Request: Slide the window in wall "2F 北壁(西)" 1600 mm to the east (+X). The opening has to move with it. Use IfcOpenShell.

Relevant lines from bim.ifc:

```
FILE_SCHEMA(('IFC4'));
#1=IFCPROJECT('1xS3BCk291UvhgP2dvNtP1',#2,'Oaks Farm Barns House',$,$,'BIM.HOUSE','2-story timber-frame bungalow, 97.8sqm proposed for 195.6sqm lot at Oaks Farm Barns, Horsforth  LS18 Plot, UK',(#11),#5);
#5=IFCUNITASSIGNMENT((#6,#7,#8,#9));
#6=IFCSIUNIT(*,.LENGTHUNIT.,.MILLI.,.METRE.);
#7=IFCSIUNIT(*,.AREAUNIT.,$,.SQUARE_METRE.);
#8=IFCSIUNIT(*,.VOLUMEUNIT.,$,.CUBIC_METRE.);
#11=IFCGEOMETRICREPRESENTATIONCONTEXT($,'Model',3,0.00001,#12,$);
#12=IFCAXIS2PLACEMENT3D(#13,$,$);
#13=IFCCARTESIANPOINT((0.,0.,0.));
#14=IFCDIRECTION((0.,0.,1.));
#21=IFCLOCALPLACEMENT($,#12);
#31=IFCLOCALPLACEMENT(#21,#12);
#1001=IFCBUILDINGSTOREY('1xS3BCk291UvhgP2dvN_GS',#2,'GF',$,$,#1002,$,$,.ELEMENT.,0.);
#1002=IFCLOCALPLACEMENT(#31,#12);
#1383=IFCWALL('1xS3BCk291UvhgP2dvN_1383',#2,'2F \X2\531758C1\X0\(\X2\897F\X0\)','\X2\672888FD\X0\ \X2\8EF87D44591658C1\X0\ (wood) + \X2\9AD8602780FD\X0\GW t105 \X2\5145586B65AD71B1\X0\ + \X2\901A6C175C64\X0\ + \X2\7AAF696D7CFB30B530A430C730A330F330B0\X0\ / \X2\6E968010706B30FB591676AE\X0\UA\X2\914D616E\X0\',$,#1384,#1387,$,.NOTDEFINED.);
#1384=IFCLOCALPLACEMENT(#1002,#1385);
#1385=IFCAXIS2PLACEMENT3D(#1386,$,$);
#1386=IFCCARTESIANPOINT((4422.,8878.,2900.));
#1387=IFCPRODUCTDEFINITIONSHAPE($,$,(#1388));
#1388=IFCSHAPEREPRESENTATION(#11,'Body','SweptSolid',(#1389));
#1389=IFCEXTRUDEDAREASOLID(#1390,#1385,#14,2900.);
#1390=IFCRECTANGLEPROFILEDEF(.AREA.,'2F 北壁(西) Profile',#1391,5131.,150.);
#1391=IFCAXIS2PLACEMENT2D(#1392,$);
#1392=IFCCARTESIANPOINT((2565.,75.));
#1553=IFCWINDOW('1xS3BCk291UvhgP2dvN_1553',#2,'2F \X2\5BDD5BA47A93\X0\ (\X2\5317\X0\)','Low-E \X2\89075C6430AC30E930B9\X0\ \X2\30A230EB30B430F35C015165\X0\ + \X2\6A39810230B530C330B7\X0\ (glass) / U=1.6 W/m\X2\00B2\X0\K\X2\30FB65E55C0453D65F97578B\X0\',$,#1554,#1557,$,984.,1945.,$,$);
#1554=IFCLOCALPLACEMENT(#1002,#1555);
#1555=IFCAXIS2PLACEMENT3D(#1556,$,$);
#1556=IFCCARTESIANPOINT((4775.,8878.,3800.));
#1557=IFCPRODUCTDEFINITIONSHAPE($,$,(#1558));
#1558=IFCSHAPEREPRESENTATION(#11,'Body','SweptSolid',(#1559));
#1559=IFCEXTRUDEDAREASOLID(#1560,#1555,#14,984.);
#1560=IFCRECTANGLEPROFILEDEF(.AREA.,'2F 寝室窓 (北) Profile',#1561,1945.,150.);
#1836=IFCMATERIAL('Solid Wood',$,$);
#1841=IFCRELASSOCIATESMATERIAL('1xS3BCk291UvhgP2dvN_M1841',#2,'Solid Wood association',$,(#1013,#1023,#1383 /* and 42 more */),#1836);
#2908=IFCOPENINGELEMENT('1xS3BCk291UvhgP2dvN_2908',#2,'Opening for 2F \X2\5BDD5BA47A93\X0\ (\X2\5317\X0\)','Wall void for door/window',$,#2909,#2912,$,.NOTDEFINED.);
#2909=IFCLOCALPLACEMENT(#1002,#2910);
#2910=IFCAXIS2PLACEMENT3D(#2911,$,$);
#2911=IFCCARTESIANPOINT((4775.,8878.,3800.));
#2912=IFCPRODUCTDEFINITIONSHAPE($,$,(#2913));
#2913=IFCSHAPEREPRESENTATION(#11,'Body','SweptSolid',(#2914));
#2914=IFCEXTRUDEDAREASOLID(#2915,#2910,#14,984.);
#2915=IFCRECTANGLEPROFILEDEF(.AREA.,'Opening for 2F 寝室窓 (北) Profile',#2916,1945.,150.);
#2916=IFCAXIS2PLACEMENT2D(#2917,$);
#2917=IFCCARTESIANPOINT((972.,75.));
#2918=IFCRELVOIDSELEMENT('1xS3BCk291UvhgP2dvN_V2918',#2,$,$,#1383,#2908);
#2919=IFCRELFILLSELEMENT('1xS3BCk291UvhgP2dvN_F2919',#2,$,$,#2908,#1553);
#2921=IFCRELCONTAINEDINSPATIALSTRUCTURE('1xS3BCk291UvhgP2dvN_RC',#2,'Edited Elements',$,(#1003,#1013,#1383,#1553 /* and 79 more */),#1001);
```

```python
import ifcopenshell
import ifcopenshell.api.geometry
import ifcopenshell.util.placement
import ifcopenshell.util.unit

model = ifcopenshell.open("bim.ifc")
unit_scale = ifcopenshell.util.unit.calculate_unit_scale(model)

window = model.by_guid("1xS3BCk291UvhgP2dvN_1553")
opening = window.FillsVoids[0].RelatingOpeningElement
wall = opening.VoidsElements[0].RelatingBuildingElement

wall_matrix = ifcopenshell.util.placement.get_local_placement(wall.ObjectPlacement)
shift = wall_matrix[:3, 0] * 1.6 / unit_scale
before = ifcopenshell.util.placement.get_local_placement(window.ObjectPlacement)[:3, 3].copy()

# The window is not placed relative to its opening, so move both.
for product in (opening, window):
    matrix = ifcopenshell.util.placement.get_local_placement(product.ObjectPlacement)
    matrix[:3, 3] += shift
    ifcopenshell.api.geometry.edit_object_placement(model, product=product, matrix=matrix, is_si=False)

after = ifcopenshell.util.placement.get_local_placement(window.ObjectPlacement)[:3, 3]
print("window moved by", (after - before).round(3) + 0.0)

model.write("bim_v2.ifc")
```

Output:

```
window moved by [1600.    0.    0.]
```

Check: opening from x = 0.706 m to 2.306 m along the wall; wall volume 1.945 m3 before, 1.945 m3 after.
